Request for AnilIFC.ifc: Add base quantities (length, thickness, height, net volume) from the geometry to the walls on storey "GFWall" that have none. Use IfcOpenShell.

First a look at what the model holds.

```python
import ifcopenshell
import ifcopenshell.util.element
import ifcopenshell.util.unit

model = ifcopenshell.open("AnilIFC.ifc")
print(model.schema)
for unit_type in ("LENGTHUNIT", "AREAUNIT", "VOLUMEUNIT"):
    print(unit_type, ifcopenshell.util.unit.calculate_unit_scale(model, unit_type))
storey = next(s for s in model.by_type("IfcBuildingStorey") if s.Name == "GFWall")
walls = [e for e in ifcopenshell.util.element.get_decomposition(storey) if e.is_a("IfcWall")]
for e in sorted(walls, key=lambda e: e.id()):
    print(e.id(), e.is_a(), e.Name, list(ifcopenshell.util.element.get_psets(e, qtos_only=True)), sep=" | ")
```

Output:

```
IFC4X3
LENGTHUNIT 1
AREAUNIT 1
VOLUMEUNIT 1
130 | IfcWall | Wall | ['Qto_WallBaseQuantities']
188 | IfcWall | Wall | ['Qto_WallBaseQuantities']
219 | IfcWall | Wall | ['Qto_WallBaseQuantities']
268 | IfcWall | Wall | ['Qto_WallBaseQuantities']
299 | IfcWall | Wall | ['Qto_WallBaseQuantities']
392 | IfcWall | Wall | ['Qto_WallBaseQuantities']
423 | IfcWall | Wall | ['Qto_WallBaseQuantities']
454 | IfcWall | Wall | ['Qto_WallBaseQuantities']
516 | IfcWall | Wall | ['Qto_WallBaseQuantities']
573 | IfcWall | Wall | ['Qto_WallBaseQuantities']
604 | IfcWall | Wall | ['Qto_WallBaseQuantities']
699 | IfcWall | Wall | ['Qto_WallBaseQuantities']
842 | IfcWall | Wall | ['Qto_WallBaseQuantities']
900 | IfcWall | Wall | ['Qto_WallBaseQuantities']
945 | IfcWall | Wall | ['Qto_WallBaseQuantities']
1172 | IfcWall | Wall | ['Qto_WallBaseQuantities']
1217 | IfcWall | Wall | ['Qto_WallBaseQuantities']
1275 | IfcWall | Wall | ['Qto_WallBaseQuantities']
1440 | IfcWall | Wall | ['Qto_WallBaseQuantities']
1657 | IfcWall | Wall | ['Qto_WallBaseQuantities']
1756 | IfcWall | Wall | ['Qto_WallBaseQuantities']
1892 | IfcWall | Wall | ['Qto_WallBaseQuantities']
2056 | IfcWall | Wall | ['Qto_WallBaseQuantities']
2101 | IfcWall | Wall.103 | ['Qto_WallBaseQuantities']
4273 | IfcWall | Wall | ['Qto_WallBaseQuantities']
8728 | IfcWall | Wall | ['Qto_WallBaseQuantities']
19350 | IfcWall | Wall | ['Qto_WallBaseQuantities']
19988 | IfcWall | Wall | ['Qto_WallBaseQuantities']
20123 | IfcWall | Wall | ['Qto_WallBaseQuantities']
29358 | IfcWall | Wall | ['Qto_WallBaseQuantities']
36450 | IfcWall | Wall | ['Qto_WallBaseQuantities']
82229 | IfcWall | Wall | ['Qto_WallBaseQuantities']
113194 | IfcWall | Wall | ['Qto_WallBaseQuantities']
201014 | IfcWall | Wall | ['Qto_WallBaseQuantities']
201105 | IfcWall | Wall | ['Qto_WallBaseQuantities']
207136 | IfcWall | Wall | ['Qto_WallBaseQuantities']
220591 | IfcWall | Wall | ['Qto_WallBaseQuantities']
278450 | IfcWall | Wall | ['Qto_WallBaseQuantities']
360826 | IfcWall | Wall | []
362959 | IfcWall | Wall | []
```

```python
import ifcopenshell
import ifcopenshell.api.pset
import ifcopenshell.geom
import ifcopenshell.util.element
import ifcopenshell.util.shape
import ifcopenshell.util.unit

model = ifcopenshell.open("AnilIFC.ifc")
unit_scale = ifcopenshell.util.unit.calculate_unit_scale(model)
volume_scale = ifcopenshell.util.unit.calculate_unit_scale(model, "VOLUMEUNIT")
settings = ifcopenshell.geom.settings()

storey = next(s for s in model.by_type("IfcBuildingStorey") if s.Name == "GFWall")
walls = [e for e in ifcopenshell.util.element.get_decomposition(storey) if e.is_a("IfcWall")]

for e in sorted(walls, key=lambda e: e.id()):
    if ifcopenshell.util.element.get_psets(e, qtos_only=True, should_inherit=False):
        continue
    # Geometry comes back in metres, in the element's own axes.
    shape = ifcopenshell.geom.create_shape(settings, e)
    values = {
        "Length": ifcopenshell.util.shape.get_x(shape.geometry) / unit_scale,
        "Width": ifcopenshell.util.shape.get_y(shape.geometry) / unit_scale,
        "Height": ifcopenshell.util.shape.get_z(shape.geometry) / unit_scale,
        "NetVolume": ifcopenshell.util.shape.get_volume(shape.geometry) / volume_scale,
    }
    qto = ifcopenshell.api.pset.add_qto(model, product=e, name="Qto_WallBaseQuantities")
    ifcopenshell.api.pset.edit_qto(model, qto=qto, properties=values)
    print(e.id(), {k: round(v, 3) for k, v in values.items()})

model.write("AnilIFC_edited.ifc")
```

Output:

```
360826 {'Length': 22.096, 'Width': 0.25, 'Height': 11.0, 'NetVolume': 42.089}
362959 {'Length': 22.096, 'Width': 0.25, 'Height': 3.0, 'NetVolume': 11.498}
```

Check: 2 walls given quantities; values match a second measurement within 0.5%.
